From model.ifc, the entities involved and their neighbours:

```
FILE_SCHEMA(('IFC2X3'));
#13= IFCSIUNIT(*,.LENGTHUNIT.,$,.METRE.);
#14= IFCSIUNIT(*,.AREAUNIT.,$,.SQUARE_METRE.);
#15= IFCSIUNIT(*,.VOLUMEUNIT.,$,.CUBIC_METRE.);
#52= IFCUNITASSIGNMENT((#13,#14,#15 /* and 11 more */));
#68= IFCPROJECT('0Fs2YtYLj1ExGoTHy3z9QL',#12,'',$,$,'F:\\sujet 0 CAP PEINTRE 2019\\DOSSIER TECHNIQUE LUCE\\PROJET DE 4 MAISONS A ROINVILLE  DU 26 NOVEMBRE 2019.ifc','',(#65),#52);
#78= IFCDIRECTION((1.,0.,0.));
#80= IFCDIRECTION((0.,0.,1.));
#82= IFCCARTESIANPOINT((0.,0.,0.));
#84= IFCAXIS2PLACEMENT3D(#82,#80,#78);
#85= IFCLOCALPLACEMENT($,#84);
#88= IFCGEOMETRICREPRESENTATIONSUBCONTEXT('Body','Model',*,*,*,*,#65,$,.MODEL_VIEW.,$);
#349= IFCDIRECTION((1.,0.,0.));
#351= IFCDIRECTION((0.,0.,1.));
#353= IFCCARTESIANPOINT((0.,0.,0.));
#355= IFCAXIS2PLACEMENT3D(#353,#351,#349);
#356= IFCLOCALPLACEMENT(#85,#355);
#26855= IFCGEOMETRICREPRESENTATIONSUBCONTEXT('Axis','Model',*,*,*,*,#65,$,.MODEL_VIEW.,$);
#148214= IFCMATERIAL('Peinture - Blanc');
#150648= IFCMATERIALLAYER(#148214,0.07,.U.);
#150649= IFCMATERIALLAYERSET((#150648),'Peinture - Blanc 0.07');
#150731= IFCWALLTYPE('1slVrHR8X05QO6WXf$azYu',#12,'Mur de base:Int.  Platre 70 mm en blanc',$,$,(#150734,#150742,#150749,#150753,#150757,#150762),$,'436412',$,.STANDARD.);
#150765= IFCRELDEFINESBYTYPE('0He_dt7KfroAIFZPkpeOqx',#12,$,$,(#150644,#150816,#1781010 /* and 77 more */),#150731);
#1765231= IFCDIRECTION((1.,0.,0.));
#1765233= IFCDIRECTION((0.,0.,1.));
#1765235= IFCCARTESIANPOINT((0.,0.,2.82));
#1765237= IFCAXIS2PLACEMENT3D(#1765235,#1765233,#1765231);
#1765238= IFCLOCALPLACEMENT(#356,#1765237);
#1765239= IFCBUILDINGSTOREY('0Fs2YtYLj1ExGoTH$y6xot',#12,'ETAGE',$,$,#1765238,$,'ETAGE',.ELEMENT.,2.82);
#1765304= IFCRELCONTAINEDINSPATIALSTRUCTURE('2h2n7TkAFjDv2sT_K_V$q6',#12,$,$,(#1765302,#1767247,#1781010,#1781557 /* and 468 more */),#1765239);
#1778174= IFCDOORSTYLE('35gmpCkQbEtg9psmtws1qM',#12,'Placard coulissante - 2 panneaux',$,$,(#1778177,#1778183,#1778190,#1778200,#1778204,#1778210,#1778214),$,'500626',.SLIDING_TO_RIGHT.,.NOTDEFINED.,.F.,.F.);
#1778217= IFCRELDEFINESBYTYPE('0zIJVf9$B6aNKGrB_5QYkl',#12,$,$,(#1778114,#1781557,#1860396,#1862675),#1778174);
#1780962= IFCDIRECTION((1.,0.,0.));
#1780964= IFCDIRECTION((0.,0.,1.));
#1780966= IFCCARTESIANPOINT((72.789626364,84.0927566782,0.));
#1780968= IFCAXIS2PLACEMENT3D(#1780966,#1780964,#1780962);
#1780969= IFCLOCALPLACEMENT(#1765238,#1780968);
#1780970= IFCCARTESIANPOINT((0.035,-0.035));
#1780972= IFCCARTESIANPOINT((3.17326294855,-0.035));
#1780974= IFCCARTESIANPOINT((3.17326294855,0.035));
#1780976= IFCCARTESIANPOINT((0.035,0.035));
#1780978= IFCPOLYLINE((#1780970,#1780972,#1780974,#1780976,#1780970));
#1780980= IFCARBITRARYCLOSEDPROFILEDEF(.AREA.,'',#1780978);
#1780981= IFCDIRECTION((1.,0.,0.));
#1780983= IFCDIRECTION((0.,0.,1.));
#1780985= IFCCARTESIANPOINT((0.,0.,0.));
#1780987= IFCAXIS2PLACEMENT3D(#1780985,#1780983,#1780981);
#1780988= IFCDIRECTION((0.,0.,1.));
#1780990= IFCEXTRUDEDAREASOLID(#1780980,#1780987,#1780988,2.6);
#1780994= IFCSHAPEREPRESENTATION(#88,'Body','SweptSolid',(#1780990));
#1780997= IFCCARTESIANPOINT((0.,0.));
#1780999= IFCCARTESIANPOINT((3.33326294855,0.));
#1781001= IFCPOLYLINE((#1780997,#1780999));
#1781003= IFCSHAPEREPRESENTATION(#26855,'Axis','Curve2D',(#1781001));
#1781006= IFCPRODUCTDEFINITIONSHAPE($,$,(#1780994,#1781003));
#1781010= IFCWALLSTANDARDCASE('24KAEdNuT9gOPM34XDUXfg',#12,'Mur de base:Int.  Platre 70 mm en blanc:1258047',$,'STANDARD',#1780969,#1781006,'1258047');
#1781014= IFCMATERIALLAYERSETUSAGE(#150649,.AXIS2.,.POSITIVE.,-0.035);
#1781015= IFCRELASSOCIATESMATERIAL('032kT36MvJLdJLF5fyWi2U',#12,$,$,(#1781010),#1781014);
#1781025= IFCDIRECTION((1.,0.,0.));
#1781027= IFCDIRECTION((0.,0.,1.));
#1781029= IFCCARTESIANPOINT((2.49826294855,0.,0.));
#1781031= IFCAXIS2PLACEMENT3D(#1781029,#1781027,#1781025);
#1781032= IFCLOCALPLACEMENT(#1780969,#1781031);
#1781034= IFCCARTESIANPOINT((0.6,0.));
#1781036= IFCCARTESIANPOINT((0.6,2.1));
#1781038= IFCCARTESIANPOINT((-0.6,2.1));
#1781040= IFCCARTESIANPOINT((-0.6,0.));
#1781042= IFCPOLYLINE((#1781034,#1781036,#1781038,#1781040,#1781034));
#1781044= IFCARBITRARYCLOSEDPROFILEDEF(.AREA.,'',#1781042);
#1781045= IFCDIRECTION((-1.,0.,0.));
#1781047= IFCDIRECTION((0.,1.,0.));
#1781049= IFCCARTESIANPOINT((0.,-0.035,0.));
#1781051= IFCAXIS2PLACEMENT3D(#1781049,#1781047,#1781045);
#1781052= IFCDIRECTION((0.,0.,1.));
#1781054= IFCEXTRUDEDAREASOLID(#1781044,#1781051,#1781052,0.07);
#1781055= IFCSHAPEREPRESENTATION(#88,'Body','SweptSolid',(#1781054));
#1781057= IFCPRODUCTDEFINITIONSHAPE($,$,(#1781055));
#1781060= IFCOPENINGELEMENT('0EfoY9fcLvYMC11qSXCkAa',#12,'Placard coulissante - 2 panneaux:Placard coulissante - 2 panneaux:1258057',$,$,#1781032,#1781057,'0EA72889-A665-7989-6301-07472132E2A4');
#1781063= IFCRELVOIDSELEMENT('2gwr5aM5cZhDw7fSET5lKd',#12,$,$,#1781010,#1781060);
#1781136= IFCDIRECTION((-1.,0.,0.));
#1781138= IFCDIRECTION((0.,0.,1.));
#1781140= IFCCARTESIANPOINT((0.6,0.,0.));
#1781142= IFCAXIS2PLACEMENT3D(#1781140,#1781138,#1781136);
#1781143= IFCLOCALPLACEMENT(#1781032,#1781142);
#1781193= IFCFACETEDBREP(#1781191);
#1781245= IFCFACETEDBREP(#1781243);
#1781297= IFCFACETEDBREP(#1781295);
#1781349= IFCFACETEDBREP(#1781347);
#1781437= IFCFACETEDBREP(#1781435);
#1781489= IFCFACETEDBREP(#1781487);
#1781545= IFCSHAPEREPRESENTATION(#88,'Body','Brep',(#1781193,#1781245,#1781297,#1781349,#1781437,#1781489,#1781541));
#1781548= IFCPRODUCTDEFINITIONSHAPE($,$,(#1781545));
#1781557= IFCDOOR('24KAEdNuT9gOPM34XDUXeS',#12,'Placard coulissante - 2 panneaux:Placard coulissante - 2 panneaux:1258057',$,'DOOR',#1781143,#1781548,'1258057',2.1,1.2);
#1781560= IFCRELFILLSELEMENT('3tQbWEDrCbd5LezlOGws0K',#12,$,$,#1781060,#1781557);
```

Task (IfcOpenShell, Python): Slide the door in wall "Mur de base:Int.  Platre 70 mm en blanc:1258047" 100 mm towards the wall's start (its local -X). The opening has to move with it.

```python
import ifcopenshell
import ifcopenshell.api.geometry
import ifcopenshell.util.placement
import ifcopenshell.util.unit

model = ifcopenshell.open("model.ifc")
unit_scale = ifcopenshell.util.unit.calculate_unit_scale(model)

door = model.by_guid("24KAEdNuT9gOPM34XDUXeS")
opening = door.FillsVoids[0].RelatingOpeningElement
wall = opening.VoidsElements[0].RelatingBuildingElement

wall_matrix = ifcopenshell.util.placement.get_local_placement(wall.ObjectPlacement)
shift = wall_matrix[:3, 0] * -0.1 / unit_scale
before = ifcopenshell.util.placement.get_local_placement(door.ObjectPlacement)[:3, 3].copy()

# The door is placed relative to its opening, so it follows when the opening moves.
matrix = ifcopenshell.util.placement.get_local_placement(opening.ObjectPlacement)
matrix[:3, 3] += shift
ifcopenshell.api.geometry.edit_object_placement(
    model, product=opening, matrix=matrix, is_si=False, should_transform_children=True
)

after = ifcopenshell.util.placement.get_local_placement(door.ObjectPlacement)[:3, 3]
print("door moved by", (after - before).round(3) + 0.0)

model.write("model_rev.ifc")
```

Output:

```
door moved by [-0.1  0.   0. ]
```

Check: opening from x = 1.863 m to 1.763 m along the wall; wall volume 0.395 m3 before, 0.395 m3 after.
